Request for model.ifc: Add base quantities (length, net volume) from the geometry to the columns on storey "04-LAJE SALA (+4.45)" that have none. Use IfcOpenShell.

First a look at what the model holds.

```python
import ifcopenshell
import ifcopenshell.util.element
import ifcopenshell.util.unit

model = ifcopenshell.open("model.ifc")
print(model.schema)
for unit_type in ("LENGTHUNIT", "AREAUNIT", "VOLUMEUNIT"):
    print(unit_type, ifcopenshell.util.unit.calculate_unit_scale(model, unit_type))
storey = next(s for s in model.by_type("IfcBuildingStorey") if s.Name == "04-LAJE SALA (+4.45)")
columns = [e for e in ifcopenshell.util.element.get_decomposition(storey) if e.is_a("IfcColumn")]
for e in sorted(columns, key=lambda e: e.id()):
    print(e.id(), e.is_a(), e.Name, list(ifcopenshell.util.element.get_psets(e, qtos_only=True)), sep=" | ")
```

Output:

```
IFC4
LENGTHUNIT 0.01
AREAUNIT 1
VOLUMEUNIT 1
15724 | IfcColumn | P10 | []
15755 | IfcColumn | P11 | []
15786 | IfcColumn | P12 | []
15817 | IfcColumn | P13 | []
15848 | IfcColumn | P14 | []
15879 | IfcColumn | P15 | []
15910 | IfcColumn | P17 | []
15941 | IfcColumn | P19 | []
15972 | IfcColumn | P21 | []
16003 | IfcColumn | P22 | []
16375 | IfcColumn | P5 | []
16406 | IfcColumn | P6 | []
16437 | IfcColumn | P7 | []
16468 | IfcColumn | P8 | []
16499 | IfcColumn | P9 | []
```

```python
import ifcopenshell
import ifcopenshell.api.pset
import ifcopenshell.geom
import ifcopenshell.util.element
import ifcopenshell.util.shape
import ifcopenshell.util.unit

model = ifcopenshell.open("model.ifc")
unit_scale = ifcopenshell.util.unit.calculate_unit_scale(model)
volume_scale = ifcopenshell.util.unit.calculate_unit_scale(model, "VOLUMEUNIT")
settings = ifcopenshell.geom.settings()

storey = next(s for s in model.by_type("IfcBuildingStorey") if s.Name == "04-LAJE SALA (+4.45)")
columns = [e for e in ifcopenshell.util.element.get_decomposition(storey) if e.is_a("IfcColumn")]

for e in sorted(columns, key=lambda e: e.id()):
    if ifcopenshell.util.element.get_psets(e, qtos_only=True, should_inherit=False):
        continue
    # Geometry comes back in metres, in the element's own axes.
    shape = ifcopenshell.geom.create_shape(settings, e)
    values = {
        "Length": ifcopenshell.util.shape.get_z(shape.geometry) / unit_scale,
        "NetVolume": ifcopenshell.util.shape.get_volume(shape.geometry) / volume_scale,
    }
    qto = ifcopenshell.api.pset.add_qto(model, product=e, name="Qto_ColumnBaseQuantities")
    ifcopenshell.api.pset.edit_qto(model, qto=qto, properties=values)
    print(e.id(), {k: round(v, 3) for k, v in values.items()})

model.write("model-out.ifc")
```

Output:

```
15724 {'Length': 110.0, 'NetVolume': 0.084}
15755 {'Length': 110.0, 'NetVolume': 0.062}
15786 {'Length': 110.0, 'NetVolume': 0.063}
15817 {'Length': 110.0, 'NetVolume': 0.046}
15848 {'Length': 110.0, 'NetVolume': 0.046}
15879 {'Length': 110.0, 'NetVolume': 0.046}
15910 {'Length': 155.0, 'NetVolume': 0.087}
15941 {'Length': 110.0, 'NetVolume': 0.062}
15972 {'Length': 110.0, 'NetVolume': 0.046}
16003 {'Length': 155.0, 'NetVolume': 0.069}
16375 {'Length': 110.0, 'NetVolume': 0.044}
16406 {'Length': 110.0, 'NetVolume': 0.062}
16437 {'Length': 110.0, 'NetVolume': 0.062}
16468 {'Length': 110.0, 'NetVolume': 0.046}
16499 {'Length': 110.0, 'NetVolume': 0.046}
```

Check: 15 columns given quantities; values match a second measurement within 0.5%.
